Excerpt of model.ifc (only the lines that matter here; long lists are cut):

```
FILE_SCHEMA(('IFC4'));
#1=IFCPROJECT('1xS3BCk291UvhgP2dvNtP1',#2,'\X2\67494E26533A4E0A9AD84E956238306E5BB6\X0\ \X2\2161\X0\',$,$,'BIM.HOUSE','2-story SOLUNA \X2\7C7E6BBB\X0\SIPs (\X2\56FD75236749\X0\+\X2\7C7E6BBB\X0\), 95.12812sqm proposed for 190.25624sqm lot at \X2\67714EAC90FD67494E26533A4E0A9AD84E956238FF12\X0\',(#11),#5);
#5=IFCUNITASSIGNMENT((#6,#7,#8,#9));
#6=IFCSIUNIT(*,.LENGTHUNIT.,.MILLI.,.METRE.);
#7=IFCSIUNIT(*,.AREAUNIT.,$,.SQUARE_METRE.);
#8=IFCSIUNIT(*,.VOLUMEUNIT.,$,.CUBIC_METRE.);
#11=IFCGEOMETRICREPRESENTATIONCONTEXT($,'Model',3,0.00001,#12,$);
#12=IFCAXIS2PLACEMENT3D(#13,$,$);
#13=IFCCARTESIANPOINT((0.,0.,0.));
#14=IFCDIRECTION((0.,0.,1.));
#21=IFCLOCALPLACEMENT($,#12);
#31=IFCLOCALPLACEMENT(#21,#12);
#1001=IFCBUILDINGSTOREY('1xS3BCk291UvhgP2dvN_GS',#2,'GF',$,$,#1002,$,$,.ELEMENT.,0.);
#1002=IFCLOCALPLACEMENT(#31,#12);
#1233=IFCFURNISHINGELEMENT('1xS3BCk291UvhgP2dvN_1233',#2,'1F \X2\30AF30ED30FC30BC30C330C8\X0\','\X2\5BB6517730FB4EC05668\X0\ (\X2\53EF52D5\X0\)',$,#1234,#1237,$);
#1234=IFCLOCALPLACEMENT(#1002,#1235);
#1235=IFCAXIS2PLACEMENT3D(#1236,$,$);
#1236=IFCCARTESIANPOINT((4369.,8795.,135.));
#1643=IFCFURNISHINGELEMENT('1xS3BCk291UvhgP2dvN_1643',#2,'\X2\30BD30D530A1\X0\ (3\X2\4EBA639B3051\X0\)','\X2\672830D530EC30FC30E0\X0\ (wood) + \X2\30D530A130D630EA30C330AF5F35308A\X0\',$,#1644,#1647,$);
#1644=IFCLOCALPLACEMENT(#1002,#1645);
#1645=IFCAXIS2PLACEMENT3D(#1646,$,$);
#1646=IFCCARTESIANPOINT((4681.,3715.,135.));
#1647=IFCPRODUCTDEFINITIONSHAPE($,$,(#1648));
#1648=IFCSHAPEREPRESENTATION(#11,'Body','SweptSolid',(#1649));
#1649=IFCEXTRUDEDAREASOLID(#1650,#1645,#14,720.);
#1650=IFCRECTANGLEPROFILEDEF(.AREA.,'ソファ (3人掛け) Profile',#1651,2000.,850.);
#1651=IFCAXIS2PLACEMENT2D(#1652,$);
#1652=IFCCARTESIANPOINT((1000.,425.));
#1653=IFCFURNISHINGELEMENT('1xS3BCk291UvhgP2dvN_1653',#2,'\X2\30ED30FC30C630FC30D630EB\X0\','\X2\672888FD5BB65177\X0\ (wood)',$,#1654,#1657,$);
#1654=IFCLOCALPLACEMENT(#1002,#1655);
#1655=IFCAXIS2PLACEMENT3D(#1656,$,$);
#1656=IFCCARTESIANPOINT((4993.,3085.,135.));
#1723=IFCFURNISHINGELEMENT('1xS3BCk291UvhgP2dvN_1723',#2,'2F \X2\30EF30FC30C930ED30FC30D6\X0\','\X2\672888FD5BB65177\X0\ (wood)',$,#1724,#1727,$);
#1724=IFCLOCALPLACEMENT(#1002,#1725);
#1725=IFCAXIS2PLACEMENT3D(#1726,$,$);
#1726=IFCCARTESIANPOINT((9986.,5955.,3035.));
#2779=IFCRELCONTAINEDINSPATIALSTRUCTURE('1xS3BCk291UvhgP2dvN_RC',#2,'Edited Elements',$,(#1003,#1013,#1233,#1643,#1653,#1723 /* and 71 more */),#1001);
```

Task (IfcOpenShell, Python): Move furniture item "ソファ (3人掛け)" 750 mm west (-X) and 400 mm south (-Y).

```python
import ifcopenshell
import ifcopenshell.api.geometry
import ifcopenshell.util.placement

model = ifcopenshell.open("model.ifc")

item = model.by_id(1643)
matrix = ifcopenshell.util.placement.get_local_placement(item.ObjectPlacement)
matrix[0, 3] -= 750.0
matrix[1, 3] -= 400.0
ifcopenshell.api.geometry.edit_object_placement(model, product=item, matrix=matrix, is_si=False)

print(ifcopenshell.util.placement.get_local_placement(item.ObjectPlacement).round(3) + 0.0)

model.write("model_rev.ifc")
```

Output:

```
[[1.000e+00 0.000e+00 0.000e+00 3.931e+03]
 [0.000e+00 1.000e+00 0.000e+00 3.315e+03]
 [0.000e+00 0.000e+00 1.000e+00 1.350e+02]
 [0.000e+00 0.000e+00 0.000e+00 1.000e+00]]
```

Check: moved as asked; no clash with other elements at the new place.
